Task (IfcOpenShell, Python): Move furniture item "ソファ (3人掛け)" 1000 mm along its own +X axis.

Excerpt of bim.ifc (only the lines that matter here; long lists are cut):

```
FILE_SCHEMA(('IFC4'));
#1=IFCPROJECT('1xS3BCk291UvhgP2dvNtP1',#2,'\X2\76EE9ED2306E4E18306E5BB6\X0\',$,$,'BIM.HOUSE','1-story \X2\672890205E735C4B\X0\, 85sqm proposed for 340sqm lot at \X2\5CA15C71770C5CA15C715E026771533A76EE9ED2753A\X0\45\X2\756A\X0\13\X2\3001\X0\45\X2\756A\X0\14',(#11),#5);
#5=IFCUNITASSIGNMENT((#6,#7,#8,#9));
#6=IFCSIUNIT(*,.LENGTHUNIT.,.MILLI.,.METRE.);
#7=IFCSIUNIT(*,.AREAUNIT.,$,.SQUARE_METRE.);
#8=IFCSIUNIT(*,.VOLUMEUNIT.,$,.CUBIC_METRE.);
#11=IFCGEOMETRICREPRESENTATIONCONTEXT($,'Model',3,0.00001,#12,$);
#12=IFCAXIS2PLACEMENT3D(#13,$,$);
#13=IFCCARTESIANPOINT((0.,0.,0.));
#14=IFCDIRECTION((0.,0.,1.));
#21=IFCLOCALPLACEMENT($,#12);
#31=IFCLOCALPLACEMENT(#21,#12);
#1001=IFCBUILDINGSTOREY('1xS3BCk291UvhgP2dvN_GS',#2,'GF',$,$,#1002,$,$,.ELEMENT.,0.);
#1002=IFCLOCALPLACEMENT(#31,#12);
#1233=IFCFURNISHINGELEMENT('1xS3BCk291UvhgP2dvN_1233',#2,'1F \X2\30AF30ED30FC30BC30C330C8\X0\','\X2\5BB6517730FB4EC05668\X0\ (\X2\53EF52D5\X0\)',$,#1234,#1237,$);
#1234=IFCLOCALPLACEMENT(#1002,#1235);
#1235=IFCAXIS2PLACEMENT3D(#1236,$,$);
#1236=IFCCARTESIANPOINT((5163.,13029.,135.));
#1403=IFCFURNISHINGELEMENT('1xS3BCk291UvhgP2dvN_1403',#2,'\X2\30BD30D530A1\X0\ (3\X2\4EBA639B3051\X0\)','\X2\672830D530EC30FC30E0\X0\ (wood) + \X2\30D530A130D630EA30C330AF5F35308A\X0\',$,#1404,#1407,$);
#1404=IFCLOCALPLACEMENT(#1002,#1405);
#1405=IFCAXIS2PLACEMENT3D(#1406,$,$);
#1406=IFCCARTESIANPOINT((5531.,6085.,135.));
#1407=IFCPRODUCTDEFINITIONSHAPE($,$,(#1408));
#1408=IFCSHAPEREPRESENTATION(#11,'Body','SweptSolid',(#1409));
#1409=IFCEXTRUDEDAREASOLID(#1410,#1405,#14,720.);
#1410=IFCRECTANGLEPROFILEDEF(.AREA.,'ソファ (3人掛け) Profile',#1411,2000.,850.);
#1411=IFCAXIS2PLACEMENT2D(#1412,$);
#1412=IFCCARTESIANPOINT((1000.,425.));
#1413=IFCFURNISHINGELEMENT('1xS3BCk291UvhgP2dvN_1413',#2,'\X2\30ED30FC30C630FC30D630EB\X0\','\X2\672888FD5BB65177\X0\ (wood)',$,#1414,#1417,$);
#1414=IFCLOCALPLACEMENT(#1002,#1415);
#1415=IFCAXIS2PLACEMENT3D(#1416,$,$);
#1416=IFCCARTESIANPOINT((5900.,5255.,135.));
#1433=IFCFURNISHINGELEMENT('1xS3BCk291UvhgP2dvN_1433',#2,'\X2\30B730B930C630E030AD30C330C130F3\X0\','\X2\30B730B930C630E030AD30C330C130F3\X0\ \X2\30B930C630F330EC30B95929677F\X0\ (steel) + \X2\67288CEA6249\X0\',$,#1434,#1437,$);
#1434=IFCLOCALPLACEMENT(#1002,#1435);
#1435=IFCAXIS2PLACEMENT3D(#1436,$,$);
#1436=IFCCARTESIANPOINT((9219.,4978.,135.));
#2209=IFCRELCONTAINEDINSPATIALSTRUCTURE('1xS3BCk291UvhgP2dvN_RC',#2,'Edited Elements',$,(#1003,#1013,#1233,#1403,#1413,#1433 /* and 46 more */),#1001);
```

```python
import ifcopenshell
import ifcopenshell.api.geometry
import ifcopenshell.util.placement
import ifcopenshell.util.unit

model = ifcopenshell.open("bim.ifc")
unit_scale = ifcopenshell.util.unit.calculate_unit_scale(model)

item = model.by_id(1403)
matrix = ifcopenshell.util.placement.get_local_placement(item.ObjectPlacement)
matrix[:3, 3] += matrix[:3, 0] * 1 / unit_scale
ifcopenshell.api.geometry.edit_object_placement(model, product=item, matrix=matrix, is_si=False)

print(ifcopenshell.util.placement.get_local_placement(item.ObjectPlacement).round(3) + 0.0)

model.write("bim_updated.ifc")
```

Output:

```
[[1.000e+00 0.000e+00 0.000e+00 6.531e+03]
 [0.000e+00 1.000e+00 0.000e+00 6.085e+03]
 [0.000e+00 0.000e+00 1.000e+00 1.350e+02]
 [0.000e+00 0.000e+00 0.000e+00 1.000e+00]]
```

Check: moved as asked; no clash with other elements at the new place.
